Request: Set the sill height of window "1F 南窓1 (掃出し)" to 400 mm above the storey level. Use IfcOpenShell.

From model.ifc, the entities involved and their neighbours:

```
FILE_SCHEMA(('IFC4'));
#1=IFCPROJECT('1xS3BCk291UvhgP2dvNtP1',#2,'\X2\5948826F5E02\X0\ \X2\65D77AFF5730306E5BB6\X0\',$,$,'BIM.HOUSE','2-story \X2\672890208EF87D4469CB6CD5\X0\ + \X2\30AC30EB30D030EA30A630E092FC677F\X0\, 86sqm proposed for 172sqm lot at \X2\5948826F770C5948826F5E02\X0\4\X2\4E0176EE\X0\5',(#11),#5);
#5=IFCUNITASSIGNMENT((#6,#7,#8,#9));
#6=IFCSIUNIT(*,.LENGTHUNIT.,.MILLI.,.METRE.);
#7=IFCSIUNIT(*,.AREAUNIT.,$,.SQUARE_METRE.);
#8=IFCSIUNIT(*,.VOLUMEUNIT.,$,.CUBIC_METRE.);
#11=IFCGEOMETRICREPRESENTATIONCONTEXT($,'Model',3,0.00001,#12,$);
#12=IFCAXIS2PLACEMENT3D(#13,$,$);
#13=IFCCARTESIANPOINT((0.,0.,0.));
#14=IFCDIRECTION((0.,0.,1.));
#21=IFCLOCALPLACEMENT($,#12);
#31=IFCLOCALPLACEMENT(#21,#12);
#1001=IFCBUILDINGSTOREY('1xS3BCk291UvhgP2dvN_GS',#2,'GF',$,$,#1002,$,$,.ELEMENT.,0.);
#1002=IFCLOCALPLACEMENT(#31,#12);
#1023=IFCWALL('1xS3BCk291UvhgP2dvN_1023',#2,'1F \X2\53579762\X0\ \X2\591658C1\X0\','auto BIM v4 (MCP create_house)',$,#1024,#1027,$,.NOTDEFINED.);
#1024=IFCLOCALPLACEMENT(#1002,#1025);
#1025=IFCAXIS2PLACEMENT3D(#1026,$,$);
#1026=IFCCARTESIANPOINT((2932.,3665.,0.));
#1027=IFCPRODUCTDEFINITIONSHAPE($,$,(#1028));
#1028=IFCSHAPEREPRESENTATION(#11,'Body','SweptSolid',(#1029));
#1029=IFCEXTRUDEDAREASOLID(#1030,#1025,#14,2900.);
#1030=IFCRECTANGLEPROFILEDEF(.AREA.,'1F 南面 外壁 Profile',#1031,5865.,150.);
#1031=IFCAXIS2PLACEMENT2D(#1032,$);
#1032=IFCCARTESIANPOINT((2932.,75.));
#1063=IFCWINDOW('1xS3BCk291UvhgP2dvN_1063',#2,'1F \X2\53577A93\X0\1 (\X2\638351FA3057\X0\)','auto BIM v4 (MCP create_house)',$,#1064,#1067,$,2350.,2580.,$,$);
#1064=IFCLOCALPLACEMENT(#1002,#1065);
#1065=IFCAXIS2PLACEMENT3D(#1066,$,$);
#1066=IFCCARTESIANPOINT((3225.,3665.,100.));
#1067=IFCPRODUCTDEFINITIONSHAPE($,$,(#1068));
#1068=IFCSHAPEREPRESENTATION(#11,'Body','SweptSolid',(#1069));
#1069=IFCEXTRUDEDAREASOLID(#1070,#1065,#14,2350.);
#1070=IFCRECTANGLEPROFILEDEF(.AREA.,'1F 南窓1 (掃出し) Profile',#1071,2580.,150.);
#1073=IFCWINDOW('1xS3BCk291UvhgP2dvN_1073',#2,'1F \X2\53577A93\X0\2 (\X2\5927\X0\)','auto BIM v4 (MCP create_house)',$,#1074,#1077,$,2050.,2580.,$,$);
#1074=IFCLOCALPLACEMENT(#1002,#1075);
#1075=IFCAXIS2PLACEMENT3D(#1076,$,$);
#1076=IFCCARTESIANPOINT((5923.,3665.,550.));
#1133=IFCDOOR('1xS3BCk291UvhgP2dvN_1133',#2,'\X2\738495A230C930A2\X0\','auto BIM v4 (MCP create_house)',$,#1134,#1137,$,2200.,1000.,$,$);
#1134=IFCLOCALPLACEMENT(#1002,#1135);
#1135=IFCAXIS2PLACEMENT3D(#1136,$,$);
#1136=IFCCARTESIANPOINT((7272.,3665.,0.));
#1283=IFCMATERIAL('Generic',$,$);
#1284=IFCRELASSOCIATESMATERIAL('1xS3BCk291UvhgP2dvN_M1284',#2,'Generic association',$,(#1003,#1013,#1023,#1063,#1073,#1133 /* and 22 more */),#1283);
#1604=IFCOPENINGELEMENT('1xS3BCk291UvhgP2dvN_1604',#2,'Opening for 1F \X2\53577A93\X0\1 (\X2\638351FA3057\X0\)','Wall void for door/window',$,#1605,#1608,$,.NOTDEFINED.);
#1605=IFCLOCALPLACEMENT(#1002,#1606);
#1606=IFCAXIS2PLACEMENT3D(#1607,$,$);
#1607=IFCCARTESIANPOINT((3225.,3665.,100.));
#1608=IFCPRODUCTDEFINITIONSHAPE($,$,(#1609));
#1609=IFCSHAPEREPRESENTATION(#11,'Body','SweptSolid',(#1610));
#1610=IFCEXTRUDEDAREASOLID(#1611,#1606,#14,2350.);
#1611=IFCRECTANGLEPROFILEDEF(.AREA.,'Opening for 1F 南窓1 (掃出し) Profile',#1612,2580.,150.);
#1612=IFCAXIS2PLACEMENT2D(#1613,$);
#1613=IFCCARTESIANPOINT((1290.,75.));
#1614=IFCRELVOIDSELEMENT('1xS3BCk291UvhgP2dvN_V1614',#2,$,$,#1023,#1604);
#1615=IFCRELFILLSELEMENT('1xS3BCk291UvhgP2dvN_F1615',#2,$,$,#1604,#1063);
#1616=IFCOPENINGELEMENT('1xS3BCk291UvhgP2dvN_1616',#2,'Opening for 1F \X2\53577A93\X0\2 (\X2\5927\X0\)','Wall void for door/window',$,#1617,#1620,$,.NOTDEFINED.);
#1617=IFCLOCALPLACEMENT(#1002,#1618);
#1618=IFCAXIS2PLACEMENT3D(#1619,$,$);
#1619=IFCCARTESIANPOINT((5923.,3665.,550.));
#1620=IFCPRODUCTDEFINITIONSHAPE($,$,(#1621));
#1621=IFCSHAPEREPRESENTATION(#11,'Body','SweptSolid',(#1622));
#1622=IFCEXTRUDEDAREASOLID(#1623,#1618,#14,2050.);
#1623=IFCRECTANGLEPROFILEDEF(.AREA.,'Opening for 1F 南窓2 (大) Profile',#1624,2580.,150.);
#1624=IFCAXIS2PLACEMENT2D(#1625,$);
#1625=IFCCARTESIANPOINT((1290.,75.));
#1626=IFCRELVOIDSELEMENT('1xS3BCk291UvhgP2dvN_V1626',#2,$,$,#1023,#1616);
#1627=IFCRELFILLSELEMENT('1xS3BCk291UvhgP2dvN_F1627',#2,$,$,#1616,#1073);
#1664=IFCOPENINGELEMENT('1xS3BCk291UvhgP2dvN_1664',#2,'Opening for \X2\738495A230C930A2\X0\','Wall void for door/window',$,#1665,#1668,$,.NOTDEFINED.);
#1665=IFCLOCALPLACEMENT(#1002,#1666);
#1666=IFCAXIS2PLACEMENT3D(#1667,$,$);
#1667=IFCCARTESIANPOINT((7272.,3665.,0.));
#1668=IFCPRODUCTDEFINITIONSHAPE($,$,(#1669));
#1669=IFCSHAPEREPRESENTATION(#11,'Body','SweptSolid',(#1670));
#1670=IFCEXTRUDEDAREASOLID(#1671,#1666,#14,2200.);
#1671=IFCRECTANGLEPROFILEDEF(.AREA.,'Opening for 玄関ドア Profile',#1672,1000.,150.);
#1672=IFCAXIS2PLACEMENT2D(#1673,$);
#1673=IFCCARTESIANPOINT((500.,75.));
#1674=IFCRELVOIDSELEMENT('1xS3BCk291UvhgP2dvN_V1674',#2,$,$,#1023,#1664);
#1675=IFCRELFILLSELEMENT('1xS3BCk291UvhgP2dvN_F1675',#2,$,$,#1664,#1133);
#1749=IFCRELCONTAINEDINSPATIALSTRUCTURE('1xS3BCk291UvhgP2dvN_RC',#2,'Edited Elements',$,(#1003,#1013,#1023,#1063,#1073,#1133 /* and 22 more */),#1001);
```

```python
import numpy as np
import ifcopenshell
import ifcopenshell.api.geometry
import ifcopenshell.geom
import ifcopenshell.util.element
import ifcopenshell.util.placement
import ifcopenshell.util.shape
import ifcopenshell.util.unit

model = ifcopenshell.open("model.ifc")
unit_scale = ifcopenshell.util.unit.calculate_unit_scale(model)

window = model.by_guid("1xS3BCk291UvhgP2dvN_1063")
opening = window.FillsVoids[0].RelatingOpeningElement
storey = ifcopenshell.util.element.get_container(window, ifc_class="IfcBuildingStorey")
level = ifcopenshell.util.placement.get_local_placement(storey.ObjectPlacement)[2, 3]

# The opening's origin need not be at the sill, so measure its lowest point.
shape = ifcopenshell.geom.create_shape(ifcopenshell.geom.settings(), opening)
bottom = ifcopenshell.util.shape.get_shape_bottom_elevation(shape, shape.geometry) / unit_scale
dz = level + 400.0 - bottom

shift = np.array([0.0, 0.0, dz])
# The window is not placed relative to its opening, so move both.
for product in (opening, window):
    matrix = ifcopenshell.util.placement.get_local_placement(product.ObjectPlacement)
    matrix[:3, 3] += shift
    ifcopenshell.api.geometry.edit_object_placement(model, product=product, matrix=matrix, is_si=False)

print(f"moved by {dz * unit_scale:+.3f} m")

model.write("model_rev.ifc")
```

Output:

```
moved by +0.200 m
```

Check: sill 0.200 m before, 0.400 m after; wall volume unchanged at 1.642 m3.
